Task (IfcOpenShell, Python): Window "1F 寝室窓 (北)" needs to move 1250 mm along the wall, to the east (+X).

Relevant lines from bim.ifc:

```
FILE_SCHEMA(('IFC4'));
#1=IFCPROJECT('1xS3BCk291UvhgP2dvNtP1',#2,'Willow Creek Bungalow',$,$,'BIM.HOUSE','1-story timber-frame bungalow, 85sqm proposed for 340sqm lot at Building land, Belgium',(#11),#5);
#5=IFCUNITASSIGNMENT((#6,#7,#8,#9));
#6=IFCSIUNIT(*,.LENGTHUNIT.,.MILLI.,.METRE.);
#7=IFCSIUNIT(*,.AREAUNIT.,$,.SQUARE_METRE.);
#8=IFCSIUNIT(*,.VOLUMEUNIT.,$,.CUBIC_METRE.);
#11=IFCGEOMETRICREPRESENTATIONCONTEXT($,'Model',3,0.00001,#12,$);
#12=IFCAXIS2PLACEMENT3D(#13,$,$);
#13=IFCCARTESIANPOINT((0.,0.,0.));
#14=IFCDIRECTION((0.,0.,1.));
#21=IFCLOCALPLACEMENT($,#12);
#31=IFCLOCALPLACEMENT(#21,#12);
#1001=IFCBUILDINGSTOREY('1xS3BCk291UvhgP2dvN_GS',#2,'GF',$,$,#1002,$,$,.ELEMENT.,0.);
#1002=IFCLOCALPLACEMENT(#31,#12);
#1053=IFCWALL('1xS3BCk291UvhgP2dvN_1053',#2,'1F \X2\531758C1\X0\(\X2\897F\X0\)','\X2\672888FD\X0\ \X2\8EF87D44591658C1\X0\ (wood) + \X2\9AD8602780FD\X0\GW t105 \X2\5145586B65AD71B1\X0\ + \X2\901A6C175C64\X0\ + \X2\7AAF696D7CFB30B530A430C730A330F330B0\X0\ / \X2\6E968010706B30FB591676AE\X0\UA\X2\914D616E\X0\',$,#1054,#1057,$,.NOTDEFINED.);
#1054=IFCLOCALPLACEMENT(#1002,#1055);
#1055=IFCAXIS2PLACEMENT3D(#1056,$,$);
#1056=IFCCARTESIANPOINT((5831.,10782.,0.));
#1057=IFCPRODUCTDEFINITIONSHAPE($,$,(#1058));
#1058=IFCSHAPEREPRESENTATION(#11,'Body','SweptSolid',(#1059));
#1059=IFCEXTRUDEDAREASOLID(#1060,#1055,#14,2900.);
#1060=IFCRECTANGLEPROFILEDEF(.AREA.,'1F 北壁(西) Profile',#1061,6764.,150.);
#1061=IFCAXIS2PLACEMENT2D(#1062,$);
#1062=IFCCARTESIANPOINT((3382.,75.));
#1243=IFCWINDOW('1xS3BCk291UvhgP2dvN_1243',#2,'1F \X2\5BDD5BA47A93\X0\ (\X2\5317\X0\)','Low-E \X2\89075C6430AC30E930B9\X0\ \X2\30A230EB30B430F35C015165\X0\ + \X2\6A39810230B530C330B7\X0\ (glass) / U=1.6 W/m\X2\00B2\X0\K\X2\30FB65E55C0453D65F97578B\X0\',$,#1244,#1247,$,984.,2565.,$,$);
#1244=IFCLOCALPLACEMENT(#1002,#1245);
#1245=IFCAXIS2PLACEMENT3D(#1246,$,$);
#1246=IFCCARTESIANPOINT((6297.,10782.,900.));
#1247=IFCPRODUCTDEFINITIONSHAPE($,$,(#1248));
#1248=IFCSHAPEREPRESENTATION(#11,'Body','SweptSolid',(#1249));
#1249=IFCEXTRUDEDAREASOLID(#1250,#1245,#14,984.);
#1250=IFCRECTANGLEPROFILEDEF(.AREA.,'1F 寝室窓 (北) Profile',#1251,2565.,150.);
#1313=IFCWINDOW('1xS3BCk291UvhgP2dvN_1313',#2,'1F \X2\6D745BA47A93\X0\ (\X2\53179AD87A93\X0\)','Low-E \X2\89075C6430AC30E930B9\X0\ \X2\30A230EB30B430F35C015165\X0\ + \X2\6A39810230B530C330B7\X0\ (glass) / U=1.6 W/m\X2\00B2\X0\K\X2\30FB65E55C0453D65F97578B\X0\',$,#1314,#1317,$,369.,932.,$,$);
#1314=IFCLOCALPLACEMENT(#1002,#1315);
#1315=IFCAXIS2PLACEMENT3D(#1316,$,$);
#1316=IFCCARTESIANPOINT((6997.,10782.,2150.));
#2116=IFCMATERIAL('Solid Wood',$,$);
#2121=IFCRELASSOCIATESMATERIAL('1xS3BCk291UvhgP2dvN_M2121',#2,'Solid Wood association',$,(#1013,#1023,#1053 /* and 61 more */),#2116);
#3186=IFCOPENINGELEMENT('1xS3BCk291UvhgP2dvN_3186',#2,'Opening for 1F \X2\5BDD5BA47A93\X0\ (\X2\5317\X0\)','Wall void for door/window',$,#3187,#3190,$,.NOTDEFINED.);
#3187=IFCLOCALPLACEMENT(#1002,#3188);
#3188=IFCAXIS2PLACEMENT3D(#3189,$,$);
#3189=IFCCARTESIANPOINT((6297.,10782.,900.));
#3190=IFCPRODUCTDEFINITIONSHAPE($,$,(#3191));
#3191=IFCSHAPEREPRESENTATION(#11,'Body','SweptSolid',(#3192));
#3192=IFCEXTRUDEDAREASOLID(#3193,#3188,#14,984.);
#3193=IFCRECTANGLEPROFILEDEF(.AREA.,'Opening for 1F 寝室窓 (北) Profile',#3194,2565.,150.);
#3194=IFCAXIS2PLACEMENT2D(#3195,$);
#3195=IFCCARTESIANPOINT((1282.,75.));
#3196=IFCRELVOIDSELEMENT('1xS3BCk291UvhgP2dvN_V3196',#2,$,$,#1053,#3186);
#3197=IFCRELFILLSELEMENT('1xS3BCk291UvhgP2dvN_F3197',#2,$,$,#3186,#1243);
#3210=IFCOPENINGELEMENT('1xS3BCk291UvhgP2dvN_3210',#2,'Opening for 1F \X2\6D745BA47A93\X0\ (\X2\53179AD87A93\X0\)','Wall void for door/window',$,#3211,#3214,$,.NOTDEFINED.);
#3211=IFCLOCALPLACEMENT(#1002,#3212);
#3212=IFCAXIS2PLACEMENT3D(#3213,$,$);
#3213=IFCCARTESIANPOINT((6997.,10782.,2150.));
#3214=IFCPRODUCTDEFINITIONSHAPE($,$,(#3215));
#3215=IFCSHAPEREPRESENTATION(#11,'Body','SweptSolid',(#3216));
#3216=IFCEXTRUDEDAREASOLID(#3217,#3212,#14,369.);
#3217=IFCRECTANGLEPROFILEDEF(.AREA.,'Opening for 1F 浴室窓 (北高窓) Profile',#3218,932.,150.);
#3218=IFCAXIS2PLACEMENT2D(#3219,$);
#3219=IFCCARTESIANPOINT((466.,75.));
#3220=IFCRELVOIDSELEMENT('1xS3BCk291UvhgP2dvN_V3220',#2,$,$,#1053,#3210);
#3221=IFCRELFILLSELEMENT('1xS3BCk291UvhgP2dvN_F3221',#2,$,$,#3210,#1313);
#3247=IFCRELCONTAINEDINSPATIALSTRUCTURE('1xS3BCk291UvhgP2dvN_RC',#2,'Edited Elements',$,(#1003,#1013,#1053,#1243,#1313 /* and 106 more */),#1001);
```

```python
import ifcopenshell
import ifcopenshell.api.geometry
import ifcopenshell.util.placement
import ifcopenshell.util.unit

model = ifcopenshell.open("bim.ifc")
unit_scale = ifcopenshell.util.unit.calculate_unit_scale(model)

window = model.by_guid("1xS3BCk291UvhgP2dvN_1243")
opening = window.FillsVoids[0].RelatingOpeningElement
wall = opening.VoidsElements[0].RelatingBuildingElement

wall_matrix = ifcopenshell.util.placement.get_local_placement(wall.ObjectPlacement)
shift = wall_matrix[:3, 0] * 1.25 / unit_scale
before = ifcopenshell.util.placement.get_local_placement(window.ObjectPlacement)[:3, 3].copy()

# The window is not placed relative to its opening, so move both.
for product in (opening, window):
    matrix = ifcopenshell.util.placement.get_local_placement(product.ObjectPlacement)
    matrix[:3, 3] += shift
    ifcopenshell.api.geometry.edit_object_placement(model, product=product, matrix=matrix, is_si=False)

after = ifcopenshell.util.placement.get_local_placement(window.ObjectPlacement)[:3, 3]
print("window moved by", (after - before).round(3) + 0.0)

model.write("bim-out.ifc")
```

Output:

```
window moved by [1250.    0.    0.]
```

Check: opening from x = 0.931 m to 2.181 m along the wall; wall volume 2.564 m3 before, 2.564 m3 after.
